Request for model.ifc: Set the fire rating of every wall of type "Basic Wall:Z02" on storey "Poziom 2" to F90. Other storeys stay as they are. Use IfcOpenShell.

First a look at what the model holds.

```python
import ifcopenshell
import ifcopenshell.util.element

model = ifcopenshell.open("model.ifc")
print(model.schema)
storey = next(s for s in model.by_type("IfcBuildingStorey") if s.Name == "Poziom 2")
walls = [e for e in ifcopenshell.util.element.get_decomposition(storey) if e.is_a("IfcWall")]
seen = {}
for e in walls:
    element_type = ifcopenshell.util.element.get_type(e)
    key = (element_type.Name if element_type != e and element_type else None, ifcopenshell.util.element.get_pset(e, "Pset_WallCommon", "FireRating"))
    seen[key] = seen.get(key, 0) + 1
for (name, value), count in sorted(seen.items(), key=str):
    print(count, "x", name, "|", value)
```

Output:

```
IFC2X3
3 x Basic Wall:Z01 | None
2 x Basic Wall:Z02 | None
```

```python
import ifcopenshell
import ifcopenshell.api.pset
import ifcopenshell.util.element

model = ifcopenshell.open("model.ifc")

storey = next(s for s in model.by_type("IfcBuildingStorey") if s.Name == "Poziom 2")
walls = [e for e in ifcopenshell.util.element.get_decomposition(storey) if e.is_a("IfcWall")]

count = 0
for e in walls:
    element_type = ifcopenshell.util.element.get_type(e)
    if element_type in (None, e) or element_type.Name != "Basic Wall:Z02":
        continue
    found = ifcopenshell.util.element.get_pset(e, "Pset_WallCommon", should_inherit=False)
    if found:
        pset = model.by_id(found["id"])
        if len(ifcopenshell.util.element.get_elements_by_pset(pset)) > 1:
            pset = ifcopenshell.api.pset.unshare_pset(model, products=[e], pset=pset)[0]
    else:
        pset = ifcopenshell.api.pset.add_pset(model, product=e, name="Pset_WallCommon")
    ifcopenshell.api.pset.edit_pset(model, pset=pset, properties={"FireRating": "F90"})
    count += 1

print(count, "walls updated")

model.write("model_updated.ifc")
```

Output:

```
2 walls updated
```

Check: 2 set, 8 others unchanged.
